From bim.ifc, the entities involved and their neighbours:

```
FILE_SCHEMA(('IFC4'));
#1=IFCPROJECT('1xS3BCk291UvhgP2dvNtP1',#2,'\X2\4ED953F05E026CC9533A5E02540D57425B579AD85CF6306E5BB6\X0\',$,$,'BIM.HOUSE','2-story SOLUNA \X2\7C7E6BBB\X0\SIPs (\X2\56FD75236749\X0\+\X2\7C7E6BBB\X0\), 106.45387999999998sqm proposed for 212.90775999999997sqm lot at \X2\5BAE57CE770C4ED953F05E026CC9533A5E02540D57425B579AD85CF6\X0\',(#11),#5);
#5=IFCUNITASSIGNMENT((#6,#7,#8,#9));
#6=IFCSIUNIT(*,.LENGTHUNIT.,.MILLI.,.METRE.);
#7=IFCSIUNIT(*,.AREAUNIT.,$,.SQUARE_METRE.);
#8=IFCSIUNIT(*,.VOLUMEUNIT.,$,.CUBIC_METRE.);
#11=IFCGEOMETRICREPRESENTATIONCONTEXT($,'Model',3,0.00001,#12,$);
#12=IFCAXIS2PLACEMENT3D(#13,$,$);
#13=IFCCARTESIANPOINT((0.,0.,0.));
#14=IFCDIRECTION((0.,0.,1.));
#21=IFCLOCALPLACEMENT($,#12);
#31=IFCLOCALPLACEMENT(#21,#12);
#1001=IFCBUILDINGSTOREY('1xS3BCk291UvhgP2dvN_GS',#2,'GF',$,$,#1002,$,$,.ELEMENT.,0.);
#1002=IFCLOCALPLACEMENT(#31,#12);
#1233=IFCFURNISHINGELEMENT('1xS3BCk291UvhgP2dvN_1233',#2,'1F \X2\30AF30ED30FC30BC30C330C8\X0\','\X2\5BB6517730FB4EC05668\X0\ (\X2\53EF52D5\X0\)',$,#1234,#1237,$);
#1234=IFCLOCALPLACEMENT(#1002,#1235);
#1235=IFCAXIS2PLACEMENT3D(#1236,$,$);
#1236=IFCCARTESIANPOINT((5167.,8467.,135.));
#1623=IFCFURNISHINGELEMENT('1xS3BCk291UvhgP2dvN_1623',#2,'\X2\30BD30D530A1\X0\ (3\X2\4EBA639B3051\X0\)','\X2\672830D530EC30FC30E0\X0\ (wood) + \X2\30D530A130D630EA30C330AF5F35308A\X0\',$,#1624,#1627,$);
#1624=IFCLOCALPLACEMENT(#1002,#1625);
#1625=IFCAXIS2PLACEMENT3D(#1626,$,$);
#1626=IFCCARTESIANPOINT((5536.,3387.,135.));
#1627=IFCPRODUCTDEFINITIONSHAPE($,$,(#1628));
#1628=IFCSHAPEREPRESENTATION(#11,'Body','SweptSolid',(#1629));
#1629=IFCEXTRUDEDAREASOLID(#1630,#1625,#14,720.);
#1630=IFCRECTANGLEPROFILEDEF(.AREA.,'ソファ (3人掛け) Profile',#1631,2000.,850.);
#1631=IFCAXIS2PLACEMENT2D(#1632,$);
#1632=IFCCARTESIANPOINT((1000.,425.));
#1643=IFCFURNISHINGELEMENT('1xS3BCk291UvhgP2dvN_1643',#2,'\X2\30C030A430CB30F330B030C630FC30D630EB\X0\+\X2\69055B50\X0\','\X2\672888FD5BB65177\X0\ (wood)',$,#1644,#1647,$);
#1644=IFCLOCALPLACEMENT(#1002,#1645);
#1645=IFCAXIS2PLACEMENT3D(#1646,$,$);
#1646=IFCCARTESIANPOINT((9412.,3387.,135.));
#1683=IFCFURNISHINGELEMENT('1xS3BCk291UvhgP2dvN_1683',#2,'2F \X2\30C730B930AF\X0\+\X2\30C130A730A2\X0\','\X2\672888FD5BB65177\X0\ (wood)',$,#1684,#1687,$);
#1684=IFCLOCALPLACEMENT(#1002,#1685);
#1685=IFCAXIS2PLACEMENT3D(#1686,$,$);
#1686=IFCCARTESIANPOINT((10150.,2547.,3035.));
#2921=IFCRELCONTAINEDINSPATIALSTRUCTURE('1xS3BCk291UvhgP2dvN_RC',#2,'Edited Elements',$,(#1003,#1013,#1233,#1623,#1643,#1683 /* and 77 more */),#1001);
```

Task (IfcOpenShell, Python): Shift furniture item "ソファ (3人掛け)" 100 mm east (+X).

```python
import ifcopenshell
import ifcopenshell.api.geometry
import ifcopenshell.util.placement
import ifcopenshell.util.unit

model = ifcopenshell.open("bim.ifc")
unit_scale = ifcopenshell.util.unit.calculate_unit_scale(model)

item = model.by_guid("1xS3BCk291UvhgP2dvN_1623")
matrix = ifcopenshell.util.placement.get_local_placement(item.ObjectPlacement)
matrix[0, 3] += 0.1 / unit_scale
ifcopenshell.api.geometry.edit_object_placement(model, product=item, matrix=matrix, is_si=False)

print(ifcopenshell.util.placement.get_local_placement(item.ObjectPlacement).round(3) + 0.0)

model.write("bim-out.ifc")
```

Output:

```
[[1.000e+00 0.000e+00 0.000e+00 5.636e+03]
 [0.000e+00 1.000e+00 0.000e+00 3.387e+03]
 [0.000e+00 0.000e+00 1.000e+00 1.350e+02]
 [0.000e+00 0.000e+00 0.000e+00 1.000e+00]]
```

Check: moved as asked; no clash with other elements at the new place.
